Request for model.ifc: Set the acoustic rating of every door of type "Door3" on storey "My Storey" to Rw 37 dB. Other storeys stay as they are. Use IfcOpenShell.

First a look at what the model holds.

```python
import ifcopenshell
import ifcopenshell.util.element

model = ifcopenshell.open("model.ifc")
print(model.schema)
storey = next(s for s in model.by_type("IfcBuildingStorey") if s.Name == "My Storey")
doors = [e for e in ifcopenshell.util.element.get_decomposition(storey) if e.is_a("IfcDoor")]
seen = {}
for e in doors:
    element_type = ifcopenshell.util.element.get_type(e)
    key = (element_type.Name if element_type != e and element_type else None, ifcopenshell.util.element.get_pset(e, "Pset_DoorCommon", "AcousticRating"))
    seen[key] = seen.get(key, 0) + 1
for (name, value), count in sorted(seen.items(), key=str):
    print(count, "x", name, "|", value)
```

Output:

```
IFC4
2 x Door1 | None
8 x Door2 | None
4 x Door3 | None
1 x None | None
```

```python
import ifcopenshell
import ifcopenshell.api.pset
import ifcopenshell.util.element

model = ifcopenshell.open("model.ifc")

storey = next(s for s in model.by_type("IfcBuildingStorey") if s.Name == "My Storey")
doors = [e for e in ifcopenshell.util.element.get_decomposition(storey) if e.is_a("IfcDoor")]

count = 0
for e in doors:
    element_type = ifcopenshell.util.element.get_type(e)
    if element_type in (None, e) or element_type.Name != "Door3":
        continue
    # add_pset returns the element's existing set when there is one.
    pset = ifcopenshell.api.pset.add_pset(model, product=e, name="Pset_DoorCommon")
    ifcopenshell.api.pset.edit_pset(model, pset=pset, properties={"AcousticRating": "Rw 37 dB"})
    count += 1

print(count, "doors updated")

model.write("model_updated.ifc")
```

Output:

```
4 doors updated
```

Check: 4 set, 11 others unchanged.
